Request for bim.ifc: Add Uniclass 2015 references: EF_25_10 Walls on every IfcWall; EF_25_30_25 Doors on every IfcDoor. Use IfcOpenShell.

First a look at what the model holds.

```python
import ifcopenshell

model = ifcopenshell.open("bim.ifc")
print(model.schema)
print("classifications:", [c.Name for c in model.by_type("IfcClassification")])
for ifc_class in ("IfcDoor", "IfcRoof", "IfcStair", "IfcWall", "IfcWindow"):
    print(ifc_class, len(model.by_type(ifc_class)))
```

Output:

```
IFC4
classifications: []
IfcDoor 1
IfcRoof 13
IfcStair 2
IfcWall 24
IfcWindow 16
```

```python
import ifcopenshell
import ifcopenshell.api.classification

model = ifcopenshell.open("bim.ifc")

system = ifcopenshell.api.classification.add_classification(model, classification="Uniclass 2015")

codes = {
    "IfcWall": ("EF_25_10", "Walls"),
    "IfcDoor": ("EF_25_30_25", "Doors"),
}
for ifc_class, (code, name) in codes.items():
    products = model.by_type(ifc_class)
    ifcopenshell.api.classification.add_reference(
        model, products=products, classification=system, identification=code, name=name
    )
    print(code, len(products))

model.write("bim_edited.ifc")
```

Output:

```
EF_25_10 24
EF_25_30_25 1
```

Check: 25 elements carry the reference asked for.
